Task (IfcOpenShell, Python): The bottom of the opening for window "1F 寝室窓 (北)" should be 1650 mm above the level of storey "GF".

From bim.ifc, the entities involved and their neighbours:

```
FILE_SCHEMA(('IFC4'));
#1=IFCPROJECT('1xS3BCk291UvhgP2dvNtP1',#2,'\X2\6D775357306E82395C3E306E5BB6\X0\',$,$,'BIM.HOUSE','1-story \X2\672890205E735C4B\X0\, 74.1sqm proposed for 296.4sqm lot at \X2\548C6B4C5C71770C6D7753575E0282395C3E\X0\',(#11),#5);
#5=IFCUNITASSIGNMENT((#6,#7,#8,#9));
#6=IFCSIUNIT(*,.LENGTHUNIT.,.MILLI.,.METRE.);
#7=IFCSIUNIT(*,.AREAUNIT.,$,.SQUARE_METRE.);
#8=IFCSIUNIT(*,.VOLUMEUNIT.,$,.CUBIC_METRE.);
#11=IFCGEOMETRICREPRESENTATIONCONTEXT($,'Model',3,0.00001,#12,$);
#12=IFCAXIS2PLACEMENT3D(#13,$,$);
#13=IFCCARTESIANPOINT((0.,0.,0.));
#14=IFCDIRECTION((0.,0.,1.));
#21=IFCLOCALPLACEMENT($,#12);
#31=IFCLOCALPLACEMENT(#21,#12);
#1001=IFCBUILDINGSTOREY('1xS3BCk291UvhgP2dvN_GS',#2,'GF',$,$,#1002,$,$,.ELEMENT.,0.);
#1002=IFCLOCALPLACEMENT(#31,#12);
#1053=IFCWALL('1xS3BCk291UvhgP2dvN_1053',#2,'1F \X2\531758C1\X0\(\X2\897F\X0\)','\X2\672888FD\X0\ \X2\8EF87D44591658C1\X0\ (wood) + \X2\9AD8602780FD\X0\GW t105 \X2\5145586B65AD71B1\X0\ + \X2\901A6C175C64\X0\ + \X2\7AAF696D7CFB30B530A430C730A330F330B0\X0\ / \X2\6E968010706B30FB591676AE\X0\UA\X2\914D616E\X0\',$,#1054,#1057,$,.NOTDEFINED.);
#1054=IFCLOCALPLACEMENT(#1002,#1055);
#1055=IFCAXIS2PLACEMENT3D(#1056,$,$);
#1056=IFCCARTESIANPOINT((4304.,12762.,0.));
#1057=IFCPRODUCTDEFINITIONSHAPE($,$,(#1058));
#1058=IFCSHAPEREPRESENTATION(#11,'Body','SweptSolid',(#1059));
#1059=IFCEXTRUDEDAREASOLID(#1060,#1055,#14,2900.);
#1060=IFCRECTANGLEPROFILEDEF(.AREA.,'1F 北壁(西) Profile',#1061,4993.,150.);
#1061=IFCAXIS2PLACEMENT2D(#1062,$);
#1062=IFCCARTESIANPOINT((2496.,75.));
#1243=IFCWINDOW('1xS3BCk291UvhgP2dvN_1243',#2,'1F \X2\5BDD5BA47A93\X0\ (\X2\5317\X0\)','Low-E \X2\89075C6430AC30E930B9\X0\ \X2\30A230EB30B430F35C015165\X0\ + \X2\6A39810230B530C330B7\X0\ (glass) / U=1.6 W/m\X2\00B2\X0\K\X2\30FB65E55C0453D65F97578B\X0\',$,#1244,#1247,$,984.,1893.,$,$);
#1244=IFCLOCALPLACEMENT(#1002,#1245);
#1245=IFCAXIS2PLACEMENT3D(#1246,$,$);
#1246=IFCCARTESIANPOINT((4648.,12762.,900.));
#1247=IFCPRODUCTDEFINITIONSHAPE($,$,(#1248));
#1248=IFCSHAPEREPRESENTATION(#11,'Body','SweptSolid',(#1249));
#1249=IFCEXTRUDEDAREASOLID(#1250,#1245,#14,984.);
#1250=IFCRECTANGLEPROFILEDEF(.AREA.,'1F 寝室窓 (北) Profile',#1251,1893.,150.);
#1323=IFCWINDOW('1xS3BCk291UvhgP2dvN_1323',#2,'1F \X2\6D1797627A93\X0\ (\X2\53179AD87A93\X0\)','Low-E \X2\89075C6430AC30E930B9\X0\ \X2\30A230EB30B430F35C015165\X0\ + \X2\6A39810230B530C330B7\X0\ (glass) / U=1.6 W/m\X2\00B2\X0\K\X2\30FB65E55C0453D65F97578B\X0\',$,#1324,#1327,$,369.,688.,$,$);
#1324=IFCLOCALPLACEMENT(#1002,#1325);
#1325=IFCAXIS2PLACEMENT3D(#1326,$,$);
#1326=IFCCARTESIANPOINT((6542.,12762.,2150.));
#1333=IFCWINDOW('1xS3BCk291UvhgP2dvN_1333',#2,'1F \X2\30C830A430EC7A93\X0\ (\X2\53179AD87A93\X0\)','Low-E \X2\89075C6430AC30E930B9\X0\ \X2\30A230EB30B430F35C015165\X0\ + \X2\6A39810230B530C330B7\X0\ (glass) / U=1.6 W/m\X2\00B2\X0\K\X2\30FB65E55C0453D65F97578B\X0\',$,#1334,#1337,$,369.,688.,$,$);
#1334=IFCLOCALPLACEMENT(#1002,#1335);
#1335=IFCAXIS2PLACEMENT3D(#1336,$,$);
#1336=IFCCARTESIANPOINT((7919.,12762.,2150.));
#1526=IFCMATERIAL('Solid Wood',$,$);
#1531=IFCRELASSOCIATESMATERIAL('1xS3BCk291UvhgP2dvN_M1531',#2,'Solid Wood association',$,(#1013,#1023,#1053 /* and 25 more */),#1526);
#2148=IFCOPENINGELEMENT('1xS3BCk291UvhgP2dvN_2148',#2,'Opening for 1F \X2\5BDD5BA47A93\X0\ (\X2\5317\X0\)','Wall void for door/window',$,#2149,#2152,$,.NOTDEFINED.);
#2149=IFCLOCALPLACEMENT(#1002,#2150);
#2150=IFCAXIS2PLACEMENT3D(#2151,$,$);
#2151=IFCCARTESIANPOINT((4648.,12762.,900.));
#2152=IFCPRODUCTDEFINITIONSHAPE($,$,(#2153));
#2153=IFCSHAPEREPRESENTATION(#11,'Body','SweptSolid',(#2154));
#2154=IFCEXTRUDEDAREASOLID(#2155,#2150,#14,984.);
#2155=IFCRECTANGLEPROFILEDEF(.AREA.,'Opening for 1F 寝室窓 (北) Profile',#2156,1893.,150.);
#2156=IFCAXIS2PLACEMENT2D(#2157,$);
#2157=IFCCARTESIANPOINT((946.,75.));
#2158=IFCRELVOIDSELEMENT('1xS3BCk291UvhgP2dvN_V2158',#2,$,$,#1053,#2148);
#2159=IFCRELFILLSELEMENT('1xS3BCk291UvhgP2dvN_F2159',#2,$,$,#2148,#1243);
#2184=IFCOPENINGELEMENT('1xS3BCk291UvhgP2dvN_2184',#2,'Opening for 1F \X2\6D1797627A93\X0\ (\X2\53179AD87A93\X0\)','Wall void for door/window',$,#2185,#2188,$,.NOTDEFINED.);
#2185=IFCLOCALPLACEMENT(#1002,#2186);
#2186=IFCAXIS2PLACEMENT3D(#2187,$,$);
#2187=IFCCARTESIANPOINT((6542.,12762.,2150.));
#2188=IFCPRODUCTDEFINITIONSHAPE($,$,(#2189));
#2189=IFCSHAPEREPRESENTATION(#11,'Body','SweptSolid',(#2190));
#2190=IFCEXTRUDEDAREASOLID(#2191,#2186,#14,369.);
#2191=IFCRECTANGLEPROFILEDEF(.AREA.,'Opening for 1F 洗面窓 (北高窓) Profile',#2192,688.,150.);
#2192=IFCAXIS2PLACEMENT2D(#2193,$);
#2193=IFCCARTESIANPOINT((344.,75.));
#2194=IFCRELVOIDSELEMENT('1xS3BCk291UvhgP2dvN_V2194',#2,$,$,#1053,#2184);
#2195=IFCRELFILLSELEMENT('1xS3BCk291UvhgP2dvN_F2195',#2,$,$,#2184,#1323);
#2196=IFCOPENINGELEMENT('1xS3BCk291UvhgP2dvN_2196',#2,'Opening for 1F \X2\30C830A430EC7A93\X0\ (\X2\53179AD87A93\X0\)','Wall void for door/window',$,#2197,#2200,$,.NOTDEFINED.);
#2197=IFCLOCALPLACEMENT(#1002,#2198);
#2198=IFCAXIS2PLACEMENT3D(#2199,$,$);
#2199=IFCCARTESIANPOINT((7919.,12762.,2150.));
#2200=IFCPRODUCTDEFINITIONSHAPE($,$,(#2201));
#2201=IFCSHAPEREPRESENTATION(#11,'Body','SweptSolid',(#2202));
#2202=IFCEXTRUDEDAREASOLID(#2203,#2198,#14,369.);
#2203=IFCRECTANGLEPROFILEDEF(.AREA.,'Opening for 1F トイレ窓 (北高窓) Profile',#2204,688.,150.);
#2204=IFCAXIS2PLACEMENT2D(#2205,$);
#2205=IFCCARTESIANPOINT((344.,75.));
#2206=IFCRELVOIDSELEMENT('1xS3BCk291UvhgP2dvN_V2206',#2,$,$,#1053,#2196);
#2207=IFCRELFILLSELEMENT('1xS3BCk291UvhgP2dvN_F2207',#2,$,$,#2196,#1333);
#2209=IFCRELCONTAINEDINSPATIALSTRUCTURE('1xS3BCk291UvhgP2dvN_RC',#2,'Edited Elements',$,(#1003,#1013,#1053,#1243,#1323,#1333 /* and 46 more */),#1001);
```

```python
import numpy as np
import ifcopenshell
import ifcopenshell.api.geometry
import ifcopenshell.geom
import ifcopenshell.util.element
import ifcopenshell.util.placement
import ifcopenshell.util.shape
import ifcopenshell.util.unit

model = ifcopenshell.open("bim.ifc")
unit_scale = ifcopenshell.util.unit.calculate_unit_scale(model)

window = model.by_guid("1xS3BCk291UvhgP2dvN_1243")
opening = window.FillsVoids[0].RelatingOpeningElement
storey = ifcopenshell.util.element.get_container(window, ifc_class="IfcBuildingStorey")
level = ifcopenshell.util.placement.get_local_placement(storey.ObjectPlacement)[2, 3]

# The opening's origin need not be at the sill, so measure its lowest point.
shape = ifcopenshell.geom.create_shape(ifcopenshell.geom.settings(), opening)
bottom = ifcopenshell.util.shape.get_shape_bottom_elevation(shape, shape.geometry) / unit_scale
dz = level + 1.65 / unit_scale - bottom

shift = np.array([0.0, 0.0, dz])
# The window is not placed relative to its opening, so move both.
for product in (opening, window):
    matrix = ifcopenshell.util.placement.get_local_placement(product.ObjectPlacement)
    matrix[:3, 3] += shift
    ifcopenshell.api.geometry.edit_object_placement(model, product=product, matrix=matrix, is_si=False)

print(f"moved by {dz * unit_scale:+.3f} m")

model.write("bim_rev.ifc")
```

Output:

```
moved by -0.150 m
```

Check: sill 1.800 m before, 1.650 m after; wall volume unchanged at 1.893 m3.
